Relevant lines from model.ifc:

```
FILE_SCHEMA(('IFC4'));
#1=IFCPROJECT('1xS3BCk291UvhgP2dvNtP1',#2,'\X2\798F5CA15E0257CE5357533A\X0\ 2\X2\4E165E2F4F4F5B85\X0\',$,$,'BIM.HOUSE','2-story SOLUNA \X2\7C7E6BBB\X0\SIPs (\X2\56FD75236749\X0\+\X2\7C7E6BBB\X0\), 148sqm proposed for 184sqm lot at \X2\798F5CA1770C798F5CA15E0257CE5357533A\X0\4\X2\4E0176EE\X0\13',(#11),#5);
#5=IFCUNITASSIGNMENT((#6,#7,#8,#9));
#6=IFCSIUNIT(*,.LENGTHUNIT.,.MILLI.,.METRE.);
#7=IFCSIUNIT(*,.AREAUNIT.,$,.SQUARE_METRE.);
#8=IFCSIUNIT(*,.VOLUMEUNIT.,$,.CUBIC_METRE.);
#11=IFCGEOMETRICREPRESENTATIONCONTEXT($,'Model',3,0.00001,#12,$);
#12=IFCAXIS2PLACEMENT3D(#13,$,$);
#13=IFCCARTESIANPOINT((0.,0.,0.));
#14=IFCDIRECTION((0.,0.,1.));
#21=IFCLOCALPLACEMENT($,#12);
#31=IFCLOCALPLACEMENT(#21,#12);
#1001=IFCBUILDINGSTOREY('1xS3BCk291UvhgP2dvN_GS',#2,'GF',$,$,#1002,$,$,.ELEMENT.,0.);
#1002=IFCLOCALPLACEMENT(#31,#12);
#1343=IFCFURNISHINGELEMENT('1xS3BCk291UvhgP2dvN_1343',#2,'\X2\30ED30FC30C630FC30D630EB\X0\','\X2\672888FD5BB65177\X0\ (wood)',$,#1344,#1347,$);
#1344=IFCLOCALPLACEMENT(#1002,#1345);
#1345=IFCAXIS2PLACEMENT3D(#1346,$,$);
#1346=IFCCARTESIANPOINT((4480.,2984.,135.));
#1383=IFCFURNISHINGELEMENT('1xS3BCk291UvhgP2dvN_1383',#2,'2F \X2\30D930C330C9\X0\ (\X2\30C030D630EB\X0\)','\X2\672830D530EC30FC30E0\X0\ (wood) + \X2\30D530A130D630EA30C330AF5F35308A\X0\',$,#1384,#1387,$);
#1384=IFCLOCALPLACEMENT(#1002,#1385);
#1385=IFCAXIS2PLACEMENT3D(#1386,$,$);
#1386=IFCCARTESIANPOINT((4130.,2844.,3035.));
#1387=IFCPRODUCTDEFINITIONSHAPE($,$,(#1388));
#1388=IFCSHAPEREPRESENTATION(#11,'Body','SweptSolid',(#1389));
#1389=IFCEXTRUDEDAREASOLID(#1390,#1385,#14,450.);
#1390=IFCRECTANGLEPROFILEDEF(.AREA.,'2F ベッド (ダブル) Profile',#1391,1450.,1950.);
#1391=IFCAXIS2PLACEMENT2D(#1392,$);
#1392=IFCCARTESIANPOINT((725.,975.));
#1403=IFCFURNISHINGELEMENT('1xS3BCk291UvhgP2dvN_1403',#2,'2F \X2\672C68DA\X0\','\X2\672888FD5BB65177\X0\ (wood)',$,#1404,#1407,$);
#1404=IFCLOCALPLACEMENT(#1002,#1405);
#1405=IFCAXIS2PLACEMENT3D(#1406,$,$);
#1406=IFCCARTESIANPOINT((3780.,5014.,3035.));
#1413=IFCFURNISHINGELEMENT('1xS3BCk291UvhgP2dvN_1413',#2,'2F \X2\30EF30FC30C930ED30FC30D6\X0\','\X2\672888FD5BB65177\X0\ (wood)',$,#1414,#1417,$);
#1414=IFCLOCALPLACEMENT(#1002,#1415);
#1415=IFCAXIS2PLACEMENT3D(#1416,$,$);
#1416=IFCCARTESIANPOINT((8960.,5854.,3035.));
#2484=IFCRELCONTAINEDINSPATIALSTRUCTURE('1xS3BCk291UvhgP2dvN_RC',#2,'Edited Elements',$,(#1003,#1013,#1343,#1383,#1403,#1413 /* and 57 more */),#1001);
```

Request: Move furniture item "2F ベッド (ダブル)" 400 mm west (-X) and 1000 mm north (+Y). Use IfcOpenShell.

```python
import ifcopenshell
import ifcopenshell.api.geometry
import ifcopenshell.util.placement

model = ifcopenshell.open("model.ifc")

item = model.by_guid("1xS3BCk291UvhgP2dvN_1383")
matrix = ifcopenshell.util.placement.get_local_placement(item.ObjectPlacement)
matrix[0, 3] -= 400.0
matrix[1, 3] += 1000.0
ifcopenshell.api.geometry.edit_object_placement(model, product=item, matrix=matrix, is_si=False)

print(ifcopenshell.util.placement.get_local_placement(item.ObjectPlacement).round(3) + 0.0)

model.write("model_updated.ifc")
```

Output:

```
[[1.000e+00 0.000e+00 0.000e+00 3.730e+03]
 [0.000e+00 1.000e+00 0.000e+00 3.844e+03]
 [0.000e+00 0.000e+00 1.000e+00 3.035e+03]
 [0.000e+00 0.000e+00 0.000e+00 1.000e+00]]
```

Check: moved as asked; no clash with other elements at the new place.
